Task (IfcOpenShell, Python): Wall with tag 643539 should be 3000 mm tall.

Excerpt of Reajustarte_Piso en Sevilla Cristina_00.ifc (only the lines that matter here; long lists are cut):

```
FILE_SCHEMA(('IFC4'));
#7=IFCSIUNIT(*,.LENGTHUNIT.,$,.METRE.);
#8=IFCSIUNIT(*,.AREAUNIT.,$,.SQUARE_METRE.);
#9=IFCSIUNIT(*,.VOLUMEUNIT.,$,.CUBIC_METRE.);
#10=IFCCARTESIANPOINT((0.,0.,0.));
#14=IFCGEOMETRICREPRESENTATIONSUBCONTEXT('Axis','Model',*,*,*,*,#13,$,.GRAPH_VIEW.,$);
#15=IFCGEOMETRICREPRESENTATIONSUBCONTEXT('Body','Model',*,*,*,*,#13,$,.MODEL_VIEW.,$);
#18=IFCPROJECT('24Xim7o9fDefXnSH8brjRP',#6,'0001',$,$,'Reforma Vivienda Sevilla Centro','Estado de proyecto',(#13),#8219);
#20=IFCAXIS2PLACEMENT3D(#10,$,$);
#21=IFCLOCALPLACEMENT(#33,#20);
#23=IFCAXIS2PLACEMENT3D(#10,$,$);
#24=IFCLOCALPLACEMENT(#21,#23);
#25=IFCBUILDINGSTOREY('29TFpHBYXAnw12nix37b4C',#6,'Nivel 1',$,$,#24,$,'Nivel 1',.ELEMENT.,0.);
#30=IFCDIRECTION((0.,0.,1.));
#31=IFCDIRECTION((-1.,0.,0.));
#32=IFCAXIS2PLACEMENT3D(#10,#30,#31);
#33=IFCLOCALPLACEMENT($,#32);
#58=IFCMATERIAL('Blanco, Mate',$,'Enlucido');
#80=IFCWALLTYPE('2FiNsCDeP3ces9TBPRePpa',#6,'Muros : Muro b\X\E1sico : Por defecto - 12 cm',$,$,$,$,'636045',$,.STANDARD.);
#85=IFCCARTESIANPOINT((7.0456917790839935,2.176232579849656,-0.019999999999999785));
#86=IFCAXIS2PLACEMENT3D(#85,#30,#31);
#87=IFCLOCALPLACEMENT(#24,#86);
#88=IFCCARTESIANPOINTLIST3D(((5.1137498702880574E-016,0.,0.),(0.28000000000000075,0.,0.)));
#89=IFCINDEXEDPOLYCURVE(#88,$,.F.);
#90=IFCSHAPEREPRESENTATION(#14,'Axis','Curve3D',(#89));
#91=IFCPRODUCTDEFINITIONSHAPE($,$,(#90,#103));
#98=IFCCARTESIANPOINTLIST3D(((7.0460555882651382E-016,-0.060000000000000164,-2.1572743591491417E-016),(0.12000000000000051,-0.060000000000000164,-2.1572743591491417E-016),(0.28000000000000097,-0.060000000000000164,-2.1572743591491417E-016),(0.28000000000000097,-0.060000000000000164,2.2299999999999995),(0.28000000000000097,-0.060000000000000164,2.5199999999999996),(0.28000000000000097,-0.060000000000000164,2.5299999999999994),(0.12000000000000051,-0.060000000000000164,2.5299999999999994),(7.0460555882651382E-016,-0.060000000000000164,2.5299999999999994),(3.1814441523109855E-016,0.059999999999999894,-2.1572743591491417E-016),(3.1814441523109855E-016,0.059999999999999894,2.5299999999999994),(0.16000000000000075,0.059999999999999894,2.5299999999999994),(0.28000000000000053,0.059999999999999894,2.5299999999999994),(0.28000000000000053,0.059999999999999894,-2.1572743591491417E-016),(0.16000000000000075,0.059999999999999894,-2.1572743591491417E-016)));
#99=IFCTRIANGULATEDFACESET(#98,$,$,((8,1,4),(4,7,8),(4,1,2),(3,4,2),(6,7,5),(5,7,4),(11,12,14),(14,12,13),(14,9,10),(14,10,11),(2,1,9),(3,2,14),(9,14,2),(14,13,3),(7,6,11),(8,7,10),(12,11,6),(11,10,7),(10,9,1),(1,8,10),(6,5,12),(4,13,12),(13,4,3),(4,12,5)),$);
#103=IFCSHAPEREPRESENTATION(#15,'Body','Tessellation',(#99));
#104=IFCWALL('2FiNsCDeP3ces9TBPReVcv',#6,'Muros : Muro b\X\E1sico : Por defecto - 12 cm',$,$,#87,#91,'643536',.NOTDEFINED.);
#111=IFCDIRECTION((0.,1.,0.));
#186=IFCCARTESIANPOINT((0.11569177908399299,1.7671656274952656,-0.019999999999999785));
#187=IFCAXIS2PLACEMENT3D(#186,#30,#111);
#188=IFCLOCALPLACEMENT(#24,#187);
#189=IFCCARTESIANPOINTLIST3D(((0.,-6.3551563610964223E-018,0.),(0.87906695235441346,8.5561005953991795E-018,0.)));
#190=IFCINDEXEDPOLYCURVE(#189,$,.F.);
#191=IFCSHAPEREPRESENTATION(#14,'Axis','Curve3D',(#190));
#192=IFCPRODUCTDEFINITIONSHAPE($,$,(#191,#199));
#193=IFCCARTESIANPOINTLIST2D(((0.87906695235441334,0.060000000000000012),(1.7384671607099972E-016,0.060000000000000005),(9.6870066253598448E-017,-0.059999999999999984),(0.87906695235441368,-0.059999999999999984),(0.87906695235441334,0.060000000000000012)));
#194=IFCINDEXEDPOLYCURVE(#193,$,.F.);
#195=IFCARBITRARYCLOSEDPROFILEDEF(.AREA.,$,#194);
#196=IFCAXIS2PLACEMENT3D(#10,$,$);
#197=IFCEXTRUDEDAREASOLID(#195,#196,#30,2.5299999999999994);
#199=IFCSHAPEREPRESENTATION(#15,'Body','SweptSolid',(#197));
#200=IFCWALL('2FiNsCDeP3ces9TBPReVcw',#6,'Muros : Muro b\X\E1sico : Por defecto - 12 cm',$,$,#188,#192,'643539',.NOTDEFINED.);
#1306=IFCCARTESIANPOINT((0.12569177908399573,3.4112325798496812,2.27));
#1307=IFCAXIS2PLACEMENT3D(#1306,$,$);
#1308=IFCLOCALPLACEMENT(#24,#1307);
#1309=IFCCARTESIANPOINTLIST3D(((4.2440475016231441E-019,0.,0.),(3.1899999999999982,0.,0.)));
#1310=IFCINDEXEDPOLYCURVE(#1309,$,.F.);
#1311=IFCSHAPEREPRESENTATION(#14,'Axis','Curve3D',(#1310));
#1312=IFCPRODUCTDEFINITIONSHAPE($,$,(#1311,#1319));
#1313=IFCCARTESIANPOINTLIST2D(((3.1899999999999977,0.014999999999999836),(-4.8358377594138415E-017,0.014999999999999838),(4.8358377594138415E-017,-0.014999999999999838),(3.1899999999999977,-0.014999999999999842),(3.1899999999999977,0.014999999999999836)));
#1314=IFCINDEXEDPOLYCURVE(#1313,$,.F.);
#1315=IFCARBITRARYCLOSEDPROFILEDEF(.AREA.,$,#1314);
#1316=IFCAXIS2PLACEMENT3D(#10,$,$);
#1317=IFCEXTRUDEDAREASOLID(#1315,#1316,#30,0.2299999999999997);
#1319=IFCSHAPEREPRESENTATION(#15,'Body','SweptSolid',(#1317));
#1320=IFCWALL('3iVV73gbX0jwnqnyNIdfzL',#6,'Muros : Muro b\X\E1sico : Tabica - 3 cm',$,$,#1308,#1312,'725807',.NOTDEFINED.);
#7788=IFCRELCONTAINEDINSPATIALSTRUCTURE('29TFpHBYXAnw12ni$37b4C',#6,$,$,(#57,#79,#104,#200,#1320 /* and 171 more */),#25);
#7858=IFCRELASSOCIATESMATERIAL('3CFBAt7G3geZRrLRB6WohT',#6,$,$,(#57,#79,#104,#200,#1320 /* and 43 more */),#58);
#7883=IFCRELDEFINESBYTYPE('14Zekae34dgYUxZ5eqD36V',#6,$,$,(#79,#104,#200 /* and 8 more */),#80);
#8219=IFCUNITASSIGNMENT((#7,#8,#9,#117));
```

```python
import ifcopenshell
import ifcopenshell.geom
import ifcopenshell.util.representation
import ifcopenshell.util.shape

model = ifcopenshell.open("Reajustarte_Piso en Sevilla Cristina_00.ifc")
settings = ifcopenshell.geom.settings()


def volume(element):
    """Net volume in cubic metres, openings subtracted."""
    shape = ifcopenshell.geom.create_shape(settings, element)
    return ifcopenshell.util.shape.get_volume(shape.geometry)


wall = model.by_guid("2FiNsCDeP3ces9TBPReVcw")
before = volume(wall)

body = ifcopenshell.util.representation.get_representation(wall, "Model", "Body")
solid = body.Items[0]
old_height = solid.Depth
solid.Depth = 3.0
after = volume(wall)

print(f"height {old_height:g} -> {solid.Depth:g}, volume {before:.3f} -> {after:.3f} m3")

model.write("Reajustarte_Piso en Sevilla Cristina_00-out.ifc")
```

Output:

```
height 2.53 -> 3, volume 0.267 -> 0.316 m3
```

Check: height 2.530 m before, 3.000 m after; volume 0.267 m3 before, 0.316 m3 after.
